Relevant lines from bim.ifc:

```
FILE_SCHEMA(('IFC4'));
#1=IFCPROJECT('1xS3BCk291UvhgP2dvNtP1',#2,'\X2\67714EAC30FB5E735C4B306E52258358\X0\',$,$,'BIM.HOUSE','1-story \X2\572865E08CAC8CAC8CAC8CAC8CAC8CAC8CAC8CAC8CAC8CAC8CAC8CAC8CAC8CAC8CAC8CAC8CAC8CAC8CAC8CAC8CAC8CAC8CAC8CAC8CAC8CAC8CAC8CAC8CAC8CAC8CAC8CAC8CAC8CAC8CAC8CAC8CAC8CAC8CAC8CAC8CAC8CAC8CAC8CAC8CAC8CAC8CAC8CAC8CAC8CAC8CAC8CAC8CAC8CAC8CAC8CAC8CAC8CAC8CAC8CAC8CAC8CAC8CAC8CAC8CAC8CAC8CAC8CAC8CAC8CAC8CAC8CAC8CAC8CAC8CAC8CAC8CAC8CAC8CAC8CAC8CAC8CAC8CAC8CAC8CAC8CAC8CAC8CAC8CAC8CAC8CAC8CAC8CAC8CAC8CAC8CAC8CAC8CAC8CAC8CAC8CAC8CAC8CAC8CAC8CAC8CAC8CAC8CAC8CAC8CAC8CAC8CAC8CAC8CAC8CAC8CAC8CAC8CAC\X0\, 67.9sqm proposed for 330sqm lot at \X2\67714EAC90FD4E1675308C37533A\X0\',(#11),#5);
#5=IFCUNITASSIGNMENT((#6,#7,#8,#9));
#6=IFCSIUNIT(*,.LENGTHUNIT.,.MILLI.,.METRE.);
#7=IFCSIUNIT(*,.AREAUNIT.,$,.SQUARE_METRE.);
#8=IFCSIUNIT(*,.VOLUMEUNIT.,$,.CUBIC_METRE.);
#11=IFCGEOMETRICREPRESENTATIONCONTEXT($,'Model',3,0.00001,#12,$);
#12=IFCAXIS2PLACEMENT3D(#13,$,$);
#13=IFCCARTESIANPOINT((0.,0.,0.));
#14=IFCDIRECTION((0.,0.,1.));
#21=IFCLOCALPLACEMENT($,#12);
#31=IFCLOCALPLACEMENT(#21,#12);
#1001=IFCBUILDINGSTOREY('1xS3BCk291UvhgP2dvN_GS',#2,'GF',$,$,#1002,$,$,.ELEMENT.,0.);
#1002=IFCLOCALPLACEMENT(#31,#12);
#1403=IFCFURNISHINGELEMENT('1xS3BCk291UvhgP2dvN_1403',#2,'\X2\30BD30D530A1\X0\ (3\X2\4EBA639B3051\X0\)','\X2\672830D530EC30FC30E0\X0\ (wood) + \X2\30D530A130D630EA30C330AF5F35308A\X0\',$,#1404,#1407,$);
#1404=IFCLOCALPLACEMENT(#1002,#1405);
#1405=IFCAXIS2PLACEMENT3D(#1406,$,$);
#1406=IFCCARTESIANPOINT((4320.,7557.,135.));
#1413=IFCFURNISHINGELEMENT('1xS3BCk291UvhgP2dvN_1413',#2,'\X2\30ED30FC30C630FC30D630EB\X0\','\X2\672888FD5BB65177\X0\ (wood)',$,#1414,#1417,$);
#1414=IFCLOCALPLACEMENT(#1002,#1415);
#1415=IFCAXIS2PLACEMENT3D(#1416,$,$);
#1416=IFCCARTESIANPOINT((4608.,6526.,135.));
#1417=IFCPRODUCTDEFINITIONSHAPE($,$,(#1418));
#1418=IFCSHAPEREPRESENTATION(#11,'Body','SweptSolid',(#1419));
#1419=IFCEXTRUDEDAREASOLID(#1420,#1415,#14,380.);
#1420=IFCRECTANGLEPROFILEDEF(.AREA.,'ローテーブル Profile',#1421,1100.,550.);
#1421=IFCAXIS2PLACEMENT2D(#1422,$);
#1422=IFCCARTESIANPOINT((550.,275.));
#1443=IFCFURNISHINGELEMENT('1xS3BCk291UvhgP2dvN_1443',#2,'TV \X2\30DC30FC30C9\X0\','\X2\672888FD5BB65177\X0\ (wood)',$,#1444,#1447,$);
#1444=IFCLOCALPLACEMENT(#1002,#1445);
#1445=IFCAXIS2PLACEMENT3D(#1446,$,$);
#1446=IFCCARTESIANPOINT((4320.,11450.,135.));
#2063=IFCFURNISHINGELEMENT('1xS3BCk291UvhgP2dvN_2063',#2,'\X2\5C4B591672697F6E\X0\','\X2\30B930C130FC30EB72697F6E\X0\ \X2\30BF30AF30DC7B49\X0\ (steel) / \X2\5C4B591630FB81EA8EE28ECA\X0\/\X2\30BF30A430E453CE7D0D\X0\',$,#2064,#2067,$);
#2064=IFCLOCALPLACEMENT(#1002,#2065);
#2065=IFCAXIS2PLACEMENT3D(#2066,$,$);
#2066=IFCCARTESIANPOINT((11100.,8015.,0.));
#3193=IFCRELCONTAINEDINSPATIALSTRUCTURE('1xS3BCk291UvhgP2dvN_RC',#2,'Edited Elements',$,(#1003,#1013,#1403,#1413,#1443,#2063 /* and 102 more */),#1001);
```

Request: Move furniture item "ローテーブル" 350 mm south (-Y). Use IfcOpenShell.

```python
import ifcopenshell
import ifcopenshell.api.geometry
import ifcopenshell.util.placement
import ifcopenshell.util.unit

model = ifcopenshell.open("bim.ifc")
unit_scale = ifcopenshell.util.unit.calculate_unit_scale(model)

item = model.by_id(1413)
matrix = ifcopenshell.util.placement.get_local_placement(item.ObjectPlacement)
matrix[1, 3] -= 0.35 / unit_scale
ifcopenshell.api.geometry.edit_object_placement(model, product=item, matrix=matrix, is_si=False)

print(ifcopenshell.util.placement.get_local_placement(item.ObjectPlacement).round(3) + 0.0)

model.write("bim-out.ifc")
```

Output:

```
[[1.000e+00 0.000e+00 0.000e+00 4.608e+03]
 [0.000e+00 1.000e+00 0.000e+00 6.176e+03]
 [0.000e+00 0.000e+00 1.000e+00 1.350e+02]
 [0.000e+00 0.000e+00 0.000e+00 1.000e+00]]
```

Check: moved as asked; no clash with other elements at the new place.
